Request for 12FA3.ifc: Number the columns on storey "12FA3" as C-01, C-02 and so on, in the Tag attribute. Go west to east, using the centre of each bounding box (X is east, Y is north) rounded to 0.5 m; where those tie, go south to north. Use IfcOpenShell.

First a look at what the model holds.

```python
import ifcopenshell
import ifcopenshell.util.element
import ifcopenshell.util.placement

model = ifcopenshell.open("12FA3.ifc")
print(model.schema)
storey = next(s for s in model.by_type("IfcBuildingStorey") if s.Name == "12FA3")
columns = [e for e in ifcopenshell.util.element.get_decomposition(storey) if e.is_a("IfcColumn")]
for e in sorted(columns, key=lambda e: e.id()):
    origin = ifcopenshell.util.placement.get_local_placement(e.ObjectPlacement)[:3, 3]
    print(e.id(), e.Tag, e.Name, origin.round(2) + 0.0, sep=" | ")
```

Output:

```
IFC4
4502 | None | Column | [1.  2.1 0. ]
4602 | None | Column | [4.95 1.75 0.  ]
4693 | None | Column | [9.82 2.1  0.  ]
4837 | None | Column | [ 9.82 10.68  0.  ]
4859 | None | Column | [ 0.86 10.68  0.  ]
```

```python
import ifcopenshell
import ifcopenshell.geom
import ifcopenshell.util.element
import ifcopenshell.util.shape

model = ifcopenshell.open("12FA3.ifc")
settings = ifcopenshell.geom.settings()
settings.set("use-world-coords", True)


def centre(element):
    shape = ifcopenshell.geom.create_shape(settings, element)
    return ifcopenshell.util.shape.get_bbox_centroid(shape.geometry)


storey = next(s for s in model.by_type("IfcBuildingStorey") if s.Name == "12FA3")
columns = [e for e in ifcopenshell.util.element.get_decomposition(storey) if e.is_a("IfcColumn")]

# Insertion points can sit at a corner or the storey origin, so sort by the geometry (in metres).
centres = {e: centre(e) for e in columns}
columns.sort(key=lambda e: (round(centres[e][0] / 0.5), centres[e][1]))

for i, e in enumerate(columns, start=1):
    number = f"C-{i:02d}"
    e.Tag = number
    print(e.id(), number)

model.write("12FA3_rev.ifc")
```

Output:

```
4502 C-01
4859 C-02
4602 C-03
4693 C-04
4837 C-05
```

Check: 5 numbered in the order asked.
